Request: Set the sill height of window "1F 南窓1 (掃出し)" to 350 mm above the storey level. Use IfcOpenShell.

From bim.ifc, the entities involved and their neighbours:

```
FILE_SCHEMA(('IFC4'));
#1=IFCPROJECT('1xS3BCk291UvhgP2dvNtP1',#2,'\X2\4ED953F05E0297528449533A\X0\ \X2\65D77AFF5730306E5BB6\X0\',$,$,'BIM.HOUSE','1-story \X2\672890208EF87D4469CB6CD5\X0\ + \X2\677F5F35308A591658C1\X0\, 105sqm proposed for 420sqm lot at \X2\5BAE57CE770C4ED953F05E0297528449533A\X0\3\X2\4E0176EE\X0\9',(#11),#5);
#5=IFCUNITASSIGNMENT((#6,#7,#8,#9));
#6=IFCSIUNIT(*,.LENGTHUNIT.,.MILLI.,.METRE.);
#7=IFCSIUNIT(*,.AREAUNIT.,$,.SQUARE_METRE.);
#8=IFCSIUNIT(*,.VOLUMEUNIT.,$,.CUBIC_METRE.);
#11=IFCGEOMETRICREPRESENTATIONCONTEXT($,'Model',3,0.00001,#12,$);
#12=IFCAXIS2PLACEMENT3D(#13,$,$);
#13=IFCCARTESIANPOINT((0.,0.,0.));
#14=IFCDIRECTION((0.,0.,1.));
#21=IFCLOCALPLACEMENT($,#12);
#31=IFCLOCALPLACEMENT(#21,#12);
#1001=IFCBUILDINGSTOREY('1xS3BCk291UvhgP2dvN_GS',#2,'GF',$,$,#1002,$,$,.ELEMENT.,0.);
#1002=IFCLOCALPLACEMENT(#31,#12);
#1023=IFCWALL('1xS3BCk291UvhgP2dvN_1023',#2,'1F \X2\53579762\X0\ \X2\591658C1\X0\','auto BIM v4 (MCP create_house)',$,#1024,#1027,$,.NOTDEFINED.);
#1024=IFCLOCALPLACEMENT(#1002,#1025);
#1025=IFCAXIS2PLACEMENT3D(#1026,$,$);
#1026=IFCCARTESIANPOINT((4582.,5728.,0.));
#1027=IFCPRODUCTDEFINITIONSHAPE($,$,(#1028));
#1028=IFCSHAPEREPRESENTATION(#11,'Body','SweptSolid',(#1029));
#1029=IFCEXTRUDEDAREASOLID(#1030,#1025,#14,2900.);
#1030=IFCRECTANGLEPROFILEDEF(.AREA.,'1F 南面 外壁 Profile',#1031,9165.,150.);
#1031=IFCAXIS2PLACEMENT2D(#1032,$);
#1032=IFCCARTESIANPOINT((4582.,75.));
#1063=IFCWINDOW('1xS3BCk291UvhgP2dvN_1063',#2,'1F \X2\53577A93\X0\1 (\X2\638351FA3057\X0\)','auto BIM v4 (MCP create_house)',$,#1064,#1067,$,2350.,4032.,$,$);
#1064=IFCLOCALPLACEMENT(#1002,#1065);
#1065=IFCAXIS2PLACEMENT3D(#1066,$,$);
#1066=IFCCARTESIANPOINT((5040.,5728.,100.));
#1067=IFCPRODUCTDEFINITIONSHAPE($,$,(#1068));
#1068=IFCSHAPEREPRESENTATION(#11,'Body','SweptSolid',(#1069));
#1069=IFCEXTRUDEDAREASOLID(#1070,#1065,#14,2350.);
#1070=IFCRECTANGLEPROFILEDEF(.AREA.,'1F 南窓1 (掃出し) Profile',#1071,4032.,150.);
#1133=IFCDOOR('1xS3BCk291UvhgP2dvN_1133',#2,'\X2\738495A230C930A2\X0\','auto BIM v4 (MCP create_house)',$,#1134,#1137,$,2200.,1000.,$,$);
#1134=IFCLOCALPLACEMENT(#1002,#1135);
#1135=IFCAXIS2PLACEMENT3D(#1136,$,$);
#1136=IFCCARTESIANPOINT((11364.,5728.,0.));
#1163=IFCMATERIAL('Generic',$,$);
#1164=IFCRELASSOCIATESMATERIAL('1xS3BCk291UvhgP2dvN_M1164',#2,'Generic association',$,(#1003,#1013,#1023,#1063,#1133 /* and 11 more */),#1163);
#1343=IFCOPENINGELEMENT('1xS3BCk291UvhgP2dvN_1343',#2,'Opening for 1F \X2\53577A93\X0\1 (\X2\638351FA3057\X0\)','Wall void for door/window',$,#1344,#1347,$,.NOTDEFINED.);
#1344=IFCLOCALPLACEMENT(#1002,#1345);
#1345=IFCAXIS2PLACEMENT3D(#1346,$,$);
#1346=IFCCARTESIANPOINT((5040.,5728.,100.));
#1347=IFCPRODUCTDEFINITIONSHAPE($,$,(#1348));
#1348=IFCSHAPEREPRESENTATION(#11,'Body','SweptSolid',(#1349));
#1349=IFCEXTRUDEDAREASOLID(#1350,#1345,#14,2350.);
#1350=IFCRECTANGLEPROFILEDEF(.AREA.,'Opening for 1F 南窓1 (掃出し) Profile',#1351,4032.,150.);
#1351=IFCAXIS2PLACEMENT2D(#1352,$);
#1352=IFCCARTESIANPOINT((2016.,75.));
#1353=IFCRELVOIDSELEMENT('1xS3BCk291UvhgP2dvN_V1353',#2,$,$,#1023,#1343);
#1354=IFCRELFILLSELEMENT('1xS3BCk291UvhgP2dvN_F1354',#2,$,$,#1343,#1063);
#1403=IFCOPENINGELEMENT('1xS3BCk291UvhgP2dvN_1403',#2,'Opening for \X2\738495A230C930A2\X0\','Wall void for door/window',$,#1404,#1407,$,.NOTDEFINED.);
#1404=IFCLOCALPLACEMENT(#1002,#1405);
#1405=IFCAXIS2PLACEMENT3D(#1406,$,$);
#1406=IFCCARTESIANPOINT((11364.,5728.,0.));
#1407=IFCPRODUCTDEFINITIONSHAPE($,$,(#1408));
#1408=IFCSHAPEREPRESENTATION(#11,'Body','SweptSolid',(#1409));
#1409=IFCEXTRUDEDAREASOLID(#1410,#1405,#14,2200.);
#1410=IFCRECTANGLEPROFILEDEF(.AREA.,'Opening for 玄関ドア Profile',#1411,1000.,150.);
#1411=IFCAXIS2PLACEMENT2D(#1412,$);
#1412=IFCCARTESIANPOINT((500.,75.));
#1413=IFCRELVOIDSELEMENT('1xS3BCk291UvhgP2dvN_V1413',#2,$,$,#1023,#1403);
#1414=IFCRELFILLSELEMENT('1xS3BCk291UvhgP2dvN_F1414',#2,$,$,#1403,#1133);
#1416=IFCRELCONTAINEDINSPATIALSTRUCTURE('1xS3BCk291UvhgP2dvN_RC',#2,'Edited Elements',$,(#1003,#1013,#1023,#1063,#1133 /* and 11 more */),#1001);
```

```python
import numpy as np
import ifcopenshell
import ifcopenshell.api.geometry
import ifcopenshell.geom
import ifcopenshell.util.element
import ifcopenshell.util.placement
import ifcopenshell.util.shape
import ifcopenshell.util.unit

model = ifcopenshell.open("bim.ifc")
unit_scale = ifcopenshell.util.unit.calculate_unit_scale(model)

window = model.by_id(1063)
opening = window.FillsVoids[0].RelatingOpeningElement
storey = ifcopenshell.util.element.get_container(window, ifc_class="IfcBuildingStorey")
level = ifcopenshell.util.placement.get_local_placement(storey.ObjectPlacement)[2, 3]

# The opening's origin need not be at the sill, so measure its lowest point.
shape = ifcopenshell.geom.create_shape(ifcopenshell.geom.settings(), opening)
bottom = ifcopenshell.util.shape.get_shape_bottom_elevation(shape, shape.geometry) / unit_scale
dz = level + 0.35 / unit_scale - bottom

shift = np.array([0.0, 0.0, dz])
# The window is not placed relative to its opening, so move both.
for product in (opening, window):
    matrix = ifcopenshell.util.placement.get_local_placement(product.ObjectPlacement)
    matrix[:3, 3] += shift
    ifcopenshell.api.geometry.edit_object_placement(model, product=product, matrix=matrix, is_si=False)

print(f"moved by {dz * unit_scale:+.3f} m")

model.write("bim_rev.ifc")
```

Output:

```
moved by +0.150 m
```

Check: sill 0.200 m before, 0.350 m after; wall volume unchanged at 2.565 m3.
